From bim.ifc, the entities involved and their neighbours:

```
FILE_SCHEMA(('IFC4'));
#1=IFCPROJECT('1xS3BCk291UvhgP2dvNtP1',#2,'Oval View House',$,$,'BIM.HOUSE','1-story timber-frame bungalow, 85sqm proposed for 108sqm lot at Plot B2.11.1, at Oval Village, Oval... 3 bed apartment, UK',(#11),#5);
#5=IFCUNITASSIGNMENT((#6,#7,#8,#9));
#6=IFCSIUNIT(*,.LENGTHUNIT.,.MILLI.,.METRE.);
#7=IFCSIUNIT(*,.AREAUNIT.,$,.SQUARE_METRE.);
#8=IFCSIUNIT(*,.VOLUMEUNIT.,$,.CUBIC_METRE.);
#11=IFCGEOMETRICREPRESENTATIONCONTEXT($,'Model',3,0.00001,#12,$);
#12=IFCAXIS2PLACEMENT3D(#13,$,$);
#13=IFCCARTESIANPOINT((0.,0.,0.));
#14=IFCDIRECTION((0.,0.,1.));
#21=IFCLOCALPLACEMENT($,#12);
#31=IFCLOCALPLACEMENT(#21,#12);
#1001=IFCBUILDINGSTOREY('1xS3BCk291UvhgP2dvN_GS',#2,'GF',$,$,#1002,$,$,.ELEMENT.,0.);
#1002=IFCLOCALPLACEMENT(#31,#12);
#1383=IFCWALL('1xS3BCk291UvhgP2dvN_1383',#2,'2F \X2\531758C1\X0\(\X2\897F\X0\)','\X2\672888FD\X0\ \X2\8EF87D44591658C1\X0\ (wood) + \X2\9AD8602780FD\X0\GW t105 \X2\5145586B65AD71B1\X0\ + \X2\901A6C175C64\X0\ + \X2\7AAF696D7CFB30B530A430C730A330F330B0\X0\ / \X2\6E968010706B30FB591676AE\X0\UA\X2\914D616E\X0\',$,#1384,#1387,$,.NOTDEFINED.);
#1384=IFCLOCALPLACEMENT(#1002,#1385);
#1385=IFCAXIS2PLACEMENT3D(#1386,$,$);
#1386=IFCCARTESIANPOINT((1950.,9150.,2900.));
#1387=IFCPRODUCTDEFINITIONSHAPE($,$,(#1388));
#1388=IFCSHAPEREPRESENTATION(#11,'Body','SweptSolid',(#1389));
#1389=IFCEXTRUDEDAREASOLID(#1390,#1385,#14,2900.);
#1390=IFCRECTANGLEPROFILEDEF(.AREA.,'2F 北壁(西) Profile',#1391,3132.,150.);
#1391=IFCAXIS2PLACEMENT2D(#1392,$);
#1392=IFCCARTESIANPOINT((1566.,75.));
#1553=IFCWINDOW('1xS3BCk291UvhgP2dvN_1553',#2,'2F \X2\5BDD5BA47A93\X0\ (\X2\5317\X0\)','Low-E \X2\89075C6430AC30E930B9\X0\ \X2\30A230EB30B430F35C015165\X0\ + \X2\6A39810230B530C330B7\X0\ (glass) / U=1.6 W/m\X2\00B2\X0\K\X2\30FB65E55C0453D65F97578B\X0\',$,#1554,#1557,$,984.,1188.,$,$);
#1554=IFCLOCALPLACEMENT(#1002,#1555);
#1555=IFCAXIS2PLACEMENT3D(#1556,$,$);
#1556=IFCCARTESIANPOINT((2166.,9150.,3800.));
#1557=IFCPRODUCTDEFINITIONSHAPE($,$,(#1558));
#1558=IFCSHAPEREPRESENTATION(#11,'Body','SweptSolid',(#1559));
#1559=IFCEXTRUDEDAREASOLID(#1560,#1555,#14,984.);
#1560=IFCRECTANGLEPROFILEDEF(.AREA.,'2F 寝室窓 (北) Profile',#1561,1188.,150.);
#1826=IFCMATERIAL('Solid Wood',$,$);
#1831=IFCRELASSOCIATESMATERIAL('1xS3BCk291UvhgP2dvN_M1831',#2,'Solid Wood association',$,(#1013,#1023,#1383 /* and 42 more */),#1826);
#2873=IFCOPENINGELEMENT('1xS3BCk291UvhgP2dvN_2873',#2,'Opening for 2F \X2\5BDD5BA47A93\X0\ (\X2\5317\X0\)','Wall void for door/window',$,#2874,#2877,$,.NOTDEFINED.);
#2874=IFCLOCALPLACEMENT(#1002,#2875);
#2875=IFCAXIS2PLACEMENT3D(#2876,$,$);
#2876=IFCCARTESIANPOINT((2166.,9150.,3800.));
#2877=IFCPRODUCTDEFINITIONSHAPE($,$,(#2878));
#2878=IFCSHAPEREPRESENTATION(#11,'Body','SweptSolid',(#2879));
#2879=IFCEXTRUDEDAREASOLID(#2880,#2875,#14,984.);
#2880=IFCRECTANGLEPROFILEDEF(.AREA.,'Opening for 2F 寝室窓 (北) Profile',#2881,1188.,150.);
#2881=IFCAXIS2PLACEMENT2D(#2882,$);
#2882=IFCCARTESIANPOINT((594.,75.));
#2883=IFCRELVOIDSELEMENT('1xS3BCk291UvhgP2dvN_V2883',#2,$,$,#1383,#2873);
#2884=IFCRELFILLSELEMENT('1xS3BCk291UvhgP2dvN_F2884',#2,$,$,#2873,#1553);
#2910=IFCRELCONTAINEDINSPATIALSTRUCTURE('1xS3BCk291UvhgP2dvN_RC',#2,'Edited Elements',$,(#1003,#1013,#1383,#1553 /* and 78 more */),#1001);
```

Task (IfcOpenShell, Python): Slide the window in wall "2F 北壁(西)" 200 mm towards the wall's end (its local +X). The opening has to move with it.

```python
import ifcopenshell
import ifcopenshell.api.geometry
import ifcopenshell.util.placement
import ifcopenshell.util.unit

model = ifcopenshell.open("bim.ifc")
unit_scale = ifcopenshell.util.unit.calculate_unit_scale(model)

window = model.by_guid("1xS3BCk291UvhgP2dvN_1553")
opening = window.FillsVoids[0].RelatingOpeningElement
wall = opening.VoidsElements[0].RelatingBuildingElement

wall_matrix = ifcopenshell.util.placement.get_local_placement(wall.ObjectPlacement)
shift = wall_matrix[:3, 0] * 0.2 / unit_scale
before = ifcopenshell.util.placement.get_local_placement(window.ObjectPlacement)[:3, 3].copy()

# The window is not placed relative to its opening, so move both.
for product in (opening, window):
    matrix = ifcopenshell.util.placement.get_local_placement(product.ObjectPlacement)
    matrix[:3, 3] += shift
    ifcopenshell.api.geometry.edit_object_placement(model, product=product, matrix=matrix, is_si=False)

after = ifcopenshell.util.placement.get_local_placement(window.ObjectPlacement)[:3, 3]
print("window moved by", (after - before).round(3) + 0.0)

model.write("bim_edited.ifc")
```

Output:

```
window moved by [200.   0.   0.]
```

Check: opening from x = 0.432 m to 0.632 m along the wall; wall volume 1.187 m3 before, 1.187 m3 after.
